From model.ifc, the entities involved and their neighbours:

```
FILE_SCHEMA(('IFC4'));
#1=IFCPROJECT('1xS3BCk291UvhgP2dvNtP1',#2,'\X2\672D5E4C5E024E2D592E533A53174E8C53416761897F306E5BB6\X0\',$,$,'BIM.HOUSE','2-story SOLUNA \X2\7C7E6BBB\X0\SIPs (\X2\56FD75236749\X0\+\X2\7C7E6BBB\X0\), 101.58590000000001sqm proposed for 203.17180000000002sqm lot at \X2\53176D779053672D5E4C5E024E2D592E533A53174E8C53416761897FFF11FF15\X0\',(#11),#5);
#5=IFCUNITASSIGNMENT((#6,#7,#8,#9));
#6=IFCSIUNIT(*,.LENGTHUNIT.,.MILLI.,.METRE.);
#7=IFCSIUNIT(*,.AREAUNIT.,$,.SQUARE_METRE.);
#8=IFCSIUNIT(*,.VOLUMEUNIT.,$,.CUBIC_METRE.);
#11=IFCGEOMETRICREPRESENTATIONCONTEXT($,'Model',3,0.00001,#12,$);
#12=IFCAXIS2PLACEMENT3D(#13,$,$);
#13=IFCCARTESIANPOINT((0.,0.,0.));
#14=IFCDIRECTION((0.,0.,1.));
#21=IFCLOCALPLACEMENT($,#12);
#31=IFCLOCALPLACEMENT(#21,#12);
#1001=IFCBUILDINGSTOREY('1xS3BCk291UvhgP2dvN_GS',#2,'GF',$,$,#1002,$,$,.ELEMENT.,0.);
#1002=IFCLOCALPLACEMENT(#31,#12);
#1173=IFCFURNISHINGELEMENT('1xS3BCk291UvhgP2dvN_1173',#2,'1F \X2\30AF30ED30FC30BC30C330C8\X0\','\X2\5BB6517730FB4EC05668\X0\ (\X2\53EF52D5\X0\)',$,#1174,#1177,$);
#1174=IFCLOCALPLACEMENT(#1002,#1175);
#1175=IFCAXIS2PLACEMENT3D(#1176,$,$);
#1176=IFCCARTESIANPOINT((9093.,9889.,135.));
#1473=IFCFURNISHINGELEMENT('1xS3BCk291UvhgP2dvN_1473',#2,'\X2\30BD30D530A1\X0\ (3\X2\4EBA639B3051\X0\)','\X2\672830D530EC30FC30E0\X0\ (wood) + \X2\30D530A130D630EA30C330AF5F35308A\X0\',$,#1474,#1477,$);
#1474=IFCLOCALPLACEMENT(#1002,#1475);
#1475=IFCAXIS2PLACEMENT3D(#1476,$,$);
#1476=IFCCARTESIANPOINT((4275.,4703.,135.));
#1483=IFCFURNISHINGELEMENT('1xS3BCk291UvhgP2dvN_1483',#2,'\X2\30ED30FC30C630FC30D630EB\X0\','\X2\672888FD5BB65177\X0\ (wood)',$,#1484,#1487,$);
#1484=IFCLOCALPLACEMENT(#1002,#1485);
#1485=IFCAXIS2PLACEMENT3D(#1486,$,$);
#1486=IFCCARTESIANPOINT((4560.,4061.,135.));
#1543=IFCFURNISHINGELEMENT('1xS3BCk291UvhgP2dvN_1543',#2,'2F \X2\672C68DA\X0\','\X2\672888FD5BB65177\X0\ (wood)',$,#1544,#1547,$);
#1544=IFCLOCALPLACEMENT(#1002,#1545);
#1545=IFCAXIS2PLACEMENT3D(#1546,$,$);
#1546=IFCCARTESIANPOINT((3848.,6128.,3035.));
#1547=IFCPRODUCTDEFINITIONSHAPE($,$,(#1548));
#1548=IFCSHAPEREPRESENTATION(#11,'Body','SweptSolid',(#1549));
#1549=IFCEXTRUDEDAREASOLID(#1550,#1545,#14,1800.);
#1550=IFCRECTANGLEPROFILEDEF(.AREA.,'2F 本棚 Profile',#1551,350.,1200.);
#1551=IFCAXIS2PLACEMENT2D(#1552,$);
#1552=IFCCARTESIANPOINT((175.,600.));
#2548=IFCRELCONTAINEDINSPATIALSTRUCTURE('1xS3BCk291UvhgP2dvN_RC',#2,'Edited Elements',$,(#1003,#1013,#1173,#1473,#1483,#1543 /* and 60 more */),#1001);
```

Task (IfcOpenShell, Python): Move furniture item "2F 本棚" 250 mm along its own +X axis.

```python
import ifcopenshell
import ifcopenshell.api.geometry
import ifcopenshell.util.placement
import ifcopenshell.util.unit

model = ifcopenshell.open("model.ifc")
unit_scale = ifcopenshell.util.unit.calculate_unit_scale(model)

item = model.by_id(1543)
matrix = ifcopenshell.util.placement.get_local_placement(item.ObjectPlacement)
matrix[:3, 3] += matrix[:3, 0] * 0.25 / unit_scale
ifcopenshell.api.geometry.edit_object_placement(model, product=item, matrix=matrix, is_si=False)

print(ifcopenshell.util.placement.get_local_placement(item.ObjectPlacement).round(3) + 0.0)

model.write("model_rev.ifc")
```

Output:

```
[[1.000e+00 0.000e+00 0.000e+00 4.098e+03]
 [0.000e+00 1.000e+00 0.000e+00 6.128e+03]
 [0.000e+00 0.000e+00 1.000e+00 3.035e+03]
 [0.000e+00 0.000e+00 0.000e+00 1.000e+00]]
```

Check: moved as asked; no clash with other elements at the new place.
